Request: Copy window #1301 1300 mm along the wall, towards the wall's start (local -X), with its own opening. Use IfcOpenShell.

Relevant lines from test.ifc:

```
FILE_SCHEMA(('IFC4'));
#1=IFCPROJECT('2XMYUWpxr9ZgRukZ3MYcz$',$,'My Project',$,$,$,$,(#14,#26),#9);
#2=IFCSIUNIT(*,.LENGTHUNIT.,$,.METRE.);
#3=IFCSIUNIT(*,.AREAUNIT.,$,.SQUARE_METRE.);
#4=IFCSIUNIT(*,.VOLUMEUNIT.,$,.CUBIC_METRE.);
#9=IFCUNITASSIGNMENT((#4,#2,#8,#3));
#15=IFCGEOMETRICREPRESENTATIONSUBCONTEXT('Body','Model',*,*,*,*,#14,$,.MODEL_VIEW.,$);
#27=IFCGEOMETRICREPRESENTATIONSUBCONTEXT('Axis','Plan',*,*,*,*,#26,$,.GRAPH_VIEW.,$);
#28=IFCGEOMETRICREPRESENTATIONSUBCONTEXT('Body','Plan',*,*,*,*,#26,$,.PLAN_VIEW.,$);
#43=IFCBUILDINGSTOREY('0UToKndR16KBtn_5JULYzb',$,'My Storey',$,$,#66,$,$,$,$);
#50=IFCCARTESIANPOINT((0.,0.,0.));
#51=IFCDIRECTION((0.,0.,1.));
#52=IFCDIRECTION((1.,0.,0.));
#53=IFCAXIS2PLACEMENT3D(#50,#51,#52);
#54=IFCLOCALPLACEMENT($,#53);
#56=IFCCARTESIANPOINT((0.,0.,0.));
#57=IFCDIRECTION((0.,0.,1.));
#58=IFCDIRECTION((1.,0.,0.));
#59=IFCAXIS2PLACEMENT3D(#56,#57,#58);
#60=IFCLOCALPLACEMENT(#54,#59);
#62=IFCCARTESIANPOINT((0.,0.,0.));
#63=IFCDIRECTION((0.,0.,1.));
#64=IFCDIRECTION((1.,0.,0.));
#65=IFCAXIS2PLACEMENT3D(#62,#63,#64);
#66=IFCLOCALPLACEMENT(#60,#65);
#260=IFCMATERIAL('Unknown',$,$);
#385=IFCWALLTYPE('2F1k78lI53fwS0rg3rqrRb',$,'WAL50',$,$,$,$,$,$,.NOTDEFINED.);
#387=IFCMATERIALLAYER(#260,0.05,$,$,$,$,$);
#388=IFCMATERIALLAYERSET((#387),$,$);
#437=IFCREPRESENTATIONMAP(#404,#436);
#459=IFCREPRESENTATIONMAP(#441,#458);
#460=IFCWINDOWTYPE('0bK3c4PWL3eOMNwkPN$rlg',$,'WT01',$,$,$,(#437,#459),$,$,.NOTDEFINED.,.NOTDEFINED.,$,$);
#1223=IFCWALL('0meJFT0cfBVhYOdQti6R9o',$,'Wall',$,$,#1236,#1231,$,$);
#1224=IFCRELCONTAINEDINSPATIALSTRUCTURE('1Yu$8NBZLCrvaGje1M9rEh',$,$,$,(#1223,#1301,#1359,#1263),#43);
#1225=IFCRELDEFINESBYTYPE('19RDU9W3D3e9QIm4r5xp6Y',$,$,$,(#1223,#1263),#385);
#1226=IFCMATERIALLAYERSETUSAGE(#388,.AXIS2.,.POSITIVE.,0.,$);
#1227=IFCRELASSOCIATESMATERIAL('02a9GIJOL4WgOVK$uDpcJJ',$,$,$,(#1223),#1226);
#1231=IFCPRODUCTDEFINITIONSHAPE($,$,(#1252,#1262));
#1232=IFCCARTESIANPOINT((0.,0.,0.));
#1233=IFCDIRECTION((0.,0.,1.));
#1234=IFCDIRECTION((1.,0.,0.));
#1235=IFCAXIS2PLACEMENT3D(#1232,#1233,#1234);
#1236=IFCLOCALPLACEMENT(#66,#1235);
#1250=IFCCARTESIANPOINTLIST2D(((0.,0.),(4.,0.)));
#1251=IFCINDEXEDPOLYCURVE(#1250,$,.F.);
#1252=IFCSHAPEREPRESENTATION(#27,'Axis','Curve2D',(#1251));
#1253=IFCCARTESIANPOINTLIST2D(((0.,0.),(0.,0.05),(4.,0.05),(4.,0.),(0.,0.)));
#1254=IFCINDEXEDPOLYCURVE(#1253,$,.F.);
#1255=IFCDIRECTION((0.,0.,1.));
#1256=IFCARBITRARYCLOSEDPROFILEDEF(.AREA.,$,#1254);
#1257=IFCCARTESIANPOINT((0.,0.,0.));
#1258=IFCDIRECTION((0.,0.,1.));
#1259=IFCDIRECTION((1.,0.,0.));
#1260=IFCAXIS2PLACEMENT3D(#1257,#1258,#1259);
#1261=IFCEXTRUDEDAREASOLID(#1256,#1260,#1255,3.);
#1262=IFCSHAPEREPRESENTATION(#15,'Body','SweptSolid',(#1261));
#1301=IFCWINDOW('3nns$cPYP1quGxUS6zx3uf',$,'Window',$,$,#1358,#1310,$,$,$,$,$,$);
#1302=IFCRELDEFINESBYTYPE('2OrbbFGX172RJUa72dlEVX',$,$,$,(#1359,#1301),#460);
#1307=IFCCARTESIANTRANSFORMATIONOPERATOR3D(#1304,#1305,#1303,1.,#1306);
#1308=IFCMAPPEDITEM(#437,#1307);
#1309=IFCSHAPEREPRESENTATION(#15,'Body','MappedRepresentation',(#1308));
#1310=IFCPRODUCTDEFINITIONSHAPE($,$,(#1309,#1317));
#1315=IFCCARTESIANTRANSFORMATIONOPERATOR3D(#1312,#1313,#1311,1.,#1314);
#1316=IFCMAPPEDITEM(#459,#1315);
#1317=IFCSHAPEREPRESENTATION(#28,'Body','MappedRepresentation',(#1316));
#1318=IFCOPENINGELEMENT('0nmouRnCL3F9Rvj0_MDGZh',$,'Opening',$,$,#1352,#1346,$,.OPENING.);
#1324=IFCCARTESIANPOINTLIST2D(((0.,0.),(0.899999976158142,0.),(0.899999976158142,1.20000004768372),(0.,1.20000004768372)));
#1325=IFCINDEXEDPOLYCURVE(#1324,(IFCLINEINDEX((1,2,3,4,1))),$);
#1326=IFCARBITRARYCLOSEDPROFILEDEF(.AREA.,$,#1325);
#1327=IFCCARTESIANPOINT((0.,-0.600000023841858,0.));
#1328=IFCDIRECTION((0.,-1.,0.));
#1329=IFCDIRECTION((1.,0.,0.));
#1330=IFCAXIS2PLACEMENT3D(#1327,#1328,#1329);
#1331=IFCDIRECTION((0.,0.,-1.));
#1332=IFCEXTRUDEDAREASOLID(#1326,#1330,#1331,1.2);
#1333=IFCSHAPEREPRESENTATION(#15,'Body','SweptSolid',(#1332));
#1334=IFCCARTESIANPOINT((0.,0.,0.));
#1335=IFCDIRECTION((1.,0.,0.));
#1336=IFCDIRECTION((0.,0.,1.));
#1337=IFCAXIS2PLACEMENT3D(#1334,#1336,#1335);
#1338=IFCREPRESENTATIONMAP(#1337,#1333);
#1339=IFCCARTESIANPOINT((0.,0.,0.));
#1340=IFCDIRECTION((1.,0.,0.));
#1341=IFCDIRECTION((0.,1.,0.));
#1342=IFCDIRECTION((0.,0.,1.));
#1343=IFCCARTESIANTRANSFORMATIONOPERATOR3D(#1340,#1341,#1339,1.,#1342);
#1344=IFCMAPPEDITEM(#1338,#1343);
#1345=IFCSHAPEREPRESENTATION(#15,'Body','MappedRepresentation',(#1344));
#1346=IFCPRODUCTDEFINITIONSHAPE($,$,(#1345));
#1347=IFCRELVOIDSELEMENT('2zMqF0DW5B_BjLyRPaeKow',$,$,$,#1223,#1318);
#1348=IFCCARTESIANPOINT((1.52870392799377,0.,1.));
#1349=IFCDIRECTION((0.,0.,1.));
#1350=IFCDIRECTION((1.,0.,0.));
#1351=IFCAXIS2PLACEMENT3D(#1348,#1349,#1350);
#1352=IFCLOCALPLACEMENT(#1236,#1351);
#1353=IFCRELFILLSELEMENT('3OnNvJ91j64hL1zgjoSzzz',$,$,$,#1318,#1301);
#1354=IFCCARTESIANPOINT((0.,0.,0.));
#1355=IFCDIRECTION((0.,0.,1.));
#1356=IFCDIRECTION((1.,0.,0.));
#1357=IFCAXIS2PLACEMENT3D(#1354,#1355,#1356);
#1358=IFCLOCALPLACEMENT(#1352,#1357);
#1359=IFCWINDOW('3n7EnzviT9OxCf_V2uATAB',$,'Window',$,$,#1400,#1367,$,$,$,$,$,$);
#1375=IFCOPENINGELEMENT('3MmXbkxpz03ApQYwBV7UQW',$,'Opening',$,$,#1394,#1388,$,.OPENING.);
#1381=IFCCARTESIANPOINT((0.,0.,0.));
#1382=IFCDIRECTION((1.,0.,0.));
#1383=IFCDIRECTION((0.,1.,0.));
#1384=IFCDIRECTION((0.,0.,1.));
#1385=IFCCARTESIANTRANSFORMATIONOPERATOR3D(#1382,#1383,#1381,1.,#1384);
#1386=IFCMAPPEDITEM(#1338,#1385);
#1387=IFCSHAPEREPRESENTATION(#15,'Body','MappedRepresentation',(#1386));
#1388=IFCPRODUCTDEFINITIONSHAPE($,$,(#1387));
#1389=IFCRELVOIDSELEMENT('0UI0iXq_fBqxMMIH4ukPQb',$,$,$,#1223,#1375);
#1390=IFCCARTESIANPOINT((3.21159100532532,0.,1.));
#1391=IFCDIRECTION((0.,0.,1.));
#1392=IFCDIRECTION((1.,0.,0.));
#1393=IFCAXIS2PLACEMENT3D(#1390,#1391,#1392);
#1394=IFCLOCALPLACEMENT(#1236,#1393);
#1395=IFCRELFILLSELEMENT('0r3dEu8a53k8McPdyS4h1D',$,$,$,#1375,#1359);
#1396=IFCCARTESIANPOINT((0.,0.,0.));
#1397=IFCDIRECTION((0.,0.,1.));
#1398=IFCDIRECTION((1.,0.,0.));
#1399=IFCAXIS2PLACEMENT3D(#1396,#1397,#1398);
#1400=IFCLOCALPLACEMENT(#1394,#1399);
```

```python
import ifcopenshell
import ifcopenshell.api.feature
import ifcopenshell.api.geometry
import ifcopenshell.api.root
import ifcopenshell.geom
import ifcopenshell.util.element
import ifcopenshell.util.placement
import ifcopenshell.util.shape
import ifcopenshell.util.unit

model = ifcopenshell.open("test.ifc")
unit_scale = ifcopenshell.util.unit.calculate_unit_scale(model)
settings = ifcopenshell.geom.settings()


def volume(element):
    """Net volume in cubic metres, openings subtracted."""
    shape = ifcopenshell.geom.create_shape(settings, element)
    return ifcopenshell.util.shape.get_volume(shape.geometry)


window = model.by_id(1301)
opening = window.FillsVoids[0].RelatingOpeningElement
wall = opening.VoidsElements[0].RelatingBuildingElement
before = volume(wall)
shift = ifcopenshell.util.placement.get_local_placement(wall.ObjectPlacement)[:3, 0] * -1.3 / unit_scale

# copy_class copies the void relationship, type, container and properties, but no geometry.
new_opening = ifcopenshell.api.root.copy_class(model, product=opening)
new_opening.Representation = ifcopenshell.util.element.copy_deep(
    model, opening.Representation, exclude=["IfcGeometricRepresentationContext", "IfcRepresentationMap"]
)
new_window = ifcopenshell.api.root.copy_class(model, product=window)
new_window.Representation = ifcopenshell.util.element.copy_deep(
    model, window.Representation, exclude=["IfcGeometricRepresentationContext", "IfcRepresentationMap"]
)
ifcopenshell.api.feature.add_filling(model, opening=new_opening, element=new_window)

for old, new in ((opening, new_opening), (window, new_window)):
    matrix = ifcopenshell.util.placement.get_local_placement(old.ObjectPlacement)
    matrix[:3, 3] += shift
    ifcopenshell.api.geometry.edit_object_placement(model, product=new, matrix=matrix, is_si=False)

after = volume(wall)

print(f"wall volume {before:.3f} -> {after:.3f} m3")

model.write("test_v2.ifc")
```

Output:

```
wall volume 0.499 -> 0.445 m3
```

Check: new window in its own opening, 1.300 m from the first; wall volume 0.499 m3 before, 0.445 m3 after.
